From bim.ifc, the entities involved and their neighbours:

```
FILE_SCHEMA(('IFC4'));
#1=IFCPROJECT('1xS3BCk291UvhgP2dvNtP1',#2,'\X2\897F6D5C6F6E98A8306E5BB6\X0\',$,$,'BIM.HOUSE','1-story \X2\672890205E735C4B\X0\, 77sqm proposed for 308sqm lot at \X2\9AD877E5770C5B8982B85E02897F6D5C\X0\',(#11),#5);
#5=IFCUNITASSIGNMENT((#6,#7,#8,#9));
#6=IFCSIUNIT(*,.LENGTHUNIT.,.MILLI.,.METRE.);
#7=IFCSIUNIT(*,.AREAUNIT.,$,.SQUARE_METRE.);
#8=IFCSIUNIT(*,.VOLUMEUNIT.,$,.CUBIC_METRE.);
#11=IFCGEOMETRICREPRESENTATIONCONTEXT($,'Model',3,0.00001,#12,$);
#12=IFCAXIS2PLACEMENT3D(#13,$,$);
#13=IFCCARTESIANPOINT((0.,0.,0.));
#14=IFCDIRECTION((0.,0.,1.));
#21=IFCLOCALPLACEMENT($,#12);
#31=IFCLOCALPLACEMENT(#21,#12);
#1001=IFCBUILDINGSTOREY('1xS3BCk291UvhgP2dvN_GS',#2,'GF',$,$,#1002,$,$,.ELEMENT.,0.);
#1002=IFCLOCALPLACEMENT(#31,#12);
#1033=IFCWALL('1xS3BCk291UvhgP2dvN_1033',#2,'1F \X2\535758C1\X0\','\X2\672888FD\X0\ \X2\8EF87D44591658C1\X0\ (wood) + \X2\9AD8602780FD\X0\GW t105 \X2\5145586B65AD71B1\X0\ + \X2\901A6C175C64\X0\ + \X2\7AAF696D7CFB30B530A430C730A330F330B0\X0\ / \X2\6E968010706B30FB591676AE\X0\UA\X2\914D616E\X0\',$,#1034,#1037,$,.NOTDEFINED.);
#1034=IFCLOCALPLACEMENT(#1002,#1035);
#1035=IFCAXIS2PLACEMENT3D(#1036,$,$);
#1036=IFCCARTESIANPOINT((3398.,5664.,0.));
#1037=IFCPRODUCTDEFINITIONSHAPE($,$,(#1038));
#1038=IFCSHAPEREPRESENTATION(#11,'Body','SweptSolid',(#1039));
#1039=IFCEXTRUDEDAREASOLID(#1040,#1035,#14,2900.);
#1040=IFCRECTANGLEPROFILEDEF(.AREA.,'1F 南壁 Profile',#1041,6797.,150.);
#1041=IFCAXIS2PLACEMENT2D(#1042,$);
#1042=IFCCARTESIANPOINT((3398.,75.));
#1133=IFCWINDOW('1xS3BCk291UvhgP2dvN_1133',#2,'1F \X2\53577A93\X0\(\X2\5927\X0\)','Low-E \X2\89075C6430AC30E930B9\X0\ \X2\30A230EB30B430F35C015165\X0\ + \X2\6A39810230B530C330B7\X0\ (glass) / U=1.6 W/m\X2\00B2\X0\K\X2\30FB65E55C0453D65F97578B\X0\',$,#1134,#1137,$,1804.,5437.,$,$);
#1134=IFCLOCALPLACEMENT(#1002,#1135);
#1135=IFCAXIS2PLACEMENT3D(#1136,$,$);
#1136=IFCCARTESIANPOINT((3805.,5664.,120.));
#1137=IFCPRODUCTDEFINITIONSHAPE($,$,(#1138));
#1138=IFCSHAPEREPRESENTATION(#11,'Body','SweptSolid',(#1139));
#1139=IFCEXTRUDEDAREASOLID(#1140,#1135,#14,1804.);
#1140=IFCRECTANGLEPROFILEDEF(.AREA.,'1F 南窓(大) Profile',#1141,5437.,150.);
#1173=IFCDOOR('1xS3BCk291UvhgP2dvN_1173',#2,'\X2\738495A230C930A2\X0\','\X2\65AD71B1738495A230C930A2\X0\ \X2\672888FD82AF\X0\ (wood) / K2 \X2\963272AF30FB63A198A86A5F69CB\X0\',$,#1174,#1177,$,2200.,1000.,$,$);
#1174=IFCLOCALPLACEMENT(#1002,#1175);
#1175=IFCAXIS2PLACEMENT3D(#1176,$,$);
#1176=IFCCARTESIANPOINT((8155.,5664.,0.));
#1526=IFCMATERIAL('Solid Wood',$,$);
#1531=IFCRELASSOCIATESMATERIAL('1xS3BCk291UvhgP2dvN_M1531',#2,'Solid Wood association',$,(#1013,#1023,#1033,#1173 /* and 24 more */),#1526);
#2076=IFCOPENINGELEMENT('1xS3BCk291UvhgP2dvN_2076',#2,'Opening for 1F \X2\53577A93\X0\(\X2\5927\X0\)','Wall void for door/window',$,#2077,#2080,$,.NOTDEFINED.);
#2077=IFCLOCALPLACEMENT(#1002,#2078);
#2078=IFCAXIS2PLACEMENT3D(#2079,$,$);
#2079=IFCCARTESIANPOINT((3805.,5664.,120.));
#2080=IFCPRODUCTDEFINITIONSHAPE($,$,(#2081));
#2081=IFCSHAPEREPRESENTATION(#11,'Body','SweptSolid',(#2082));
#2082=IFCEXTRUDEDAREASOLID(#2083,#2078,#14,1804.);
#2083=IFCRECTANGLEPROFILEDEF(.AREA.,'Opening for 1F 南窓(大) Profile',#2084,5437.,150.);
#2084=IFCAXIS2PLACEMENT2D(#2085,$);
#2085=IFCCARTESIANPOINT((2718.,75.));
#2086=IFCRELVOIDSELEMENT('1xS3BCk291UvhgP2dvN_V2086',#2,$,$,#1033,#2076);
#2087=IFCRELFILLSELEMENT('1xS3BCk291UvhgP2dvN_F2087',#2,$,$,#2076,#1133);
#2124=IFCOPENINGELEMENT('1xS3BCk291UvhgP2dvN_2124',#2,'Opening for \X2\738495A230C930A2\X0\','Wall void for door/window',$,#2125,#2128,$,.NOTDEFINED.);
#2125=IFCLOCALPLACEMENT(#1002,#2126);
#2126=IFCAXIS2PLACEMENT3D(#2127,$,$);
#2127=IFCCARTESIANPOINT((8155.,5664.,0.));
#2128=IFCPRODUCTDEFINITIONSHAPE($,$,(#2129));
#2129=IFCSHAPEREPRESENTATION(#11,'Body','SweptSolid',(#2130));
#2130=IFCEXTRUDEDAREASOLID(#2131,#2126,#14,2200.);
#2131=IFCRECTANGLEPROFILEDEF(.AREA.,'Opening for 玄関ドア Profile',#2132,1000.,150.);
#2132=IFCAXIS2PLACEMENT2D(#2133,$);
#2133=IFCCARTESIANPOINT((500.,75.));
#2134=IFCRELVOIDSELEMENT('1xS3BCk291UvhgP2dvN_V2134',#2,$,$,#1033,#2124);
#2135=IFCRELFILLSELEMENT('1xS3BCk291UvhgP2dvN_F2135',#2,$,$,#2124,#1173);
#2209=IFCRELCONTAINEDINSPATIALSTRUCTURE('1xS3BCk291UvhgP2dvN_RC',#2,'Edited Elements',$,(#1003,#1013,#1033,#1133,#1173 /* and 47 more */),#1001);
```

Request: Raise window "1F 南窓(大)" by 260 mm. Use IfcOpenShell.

```python
import numpy as np
import ifcopenshell
import ifcopenshell.api.geometry
import ifcopenshell.util.placement
import ifcopenshell.util.unit

model = ifcopenshell.open("bim.ifc")
unit_scale = ifcopenshell.util.unit.calculate_unit_scale(model)

window = model.by_guid("1xS3BCk291UvhgP2dvN_1133")
opening = window.FillsVoids[0].RelatingOpeningElement
dz = 260.0

shift = np.array([0.0, 0.0, dz])
# The window is not placed relative to its opening, so move both.
for product in (opening, window):
    matrix = ifcopenshell.util.placement.get_local_placement(product.ObjectPlacement)
    matrix[:3, 3] += shift
    ifcopenshell.api.geometry.edit_object_placement(model, product=product, matrix=matrix, is_si=False)

print(f"moved by {dz * unit_scale:+.3f} m")

model.write("bim-out.ifc")
```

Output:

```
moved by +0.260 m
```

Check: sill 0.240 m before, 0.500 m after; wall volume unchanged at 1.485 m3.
